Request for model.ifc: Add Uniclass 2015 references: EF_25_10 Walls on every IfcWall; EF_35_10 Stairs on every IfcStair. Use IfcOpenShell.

First a look at what the model holds.

```python
import ifcopenshell

model = ifcopenshell.open("model.ifc")
print(model.schema)
print("classifications:", [c.Name for c in model.by_type("IfcClassification")])
for ifc_class in ("IfcDoor", "IfcRoof", "IfcStair", "IfcWall", "IfcWindow"):
    print(ifc_class, len(model.by_type(ifc_class)))
```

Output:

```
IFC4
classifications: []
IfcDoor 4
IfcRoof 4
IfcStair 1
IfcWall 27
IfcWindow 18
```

```python
import ifcopenshell
import ifcopenshell.api.classification

model = ifcopenshell.open("model.ifc")

system = ifcopenshell.api.classification.add_classification(model, classification="Uniclass 2015")

codes = {
    "IfcWall": ("EF_25_10", "Walls"),
    "IfcStair": ("EF_35_10", "Stairs"),
}
for ifc_class, (code, name) in codes.items():
    products = model.by_type(ifc_class)
    ifcopenshell.api.classification.add_reference(
        model, products=products, classification=system, identification=code, name=name
    )
    print(code, len(products))

model.write("model_v2.ifc")
```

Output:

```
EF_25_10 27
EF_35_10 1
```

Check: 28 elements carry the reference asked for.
